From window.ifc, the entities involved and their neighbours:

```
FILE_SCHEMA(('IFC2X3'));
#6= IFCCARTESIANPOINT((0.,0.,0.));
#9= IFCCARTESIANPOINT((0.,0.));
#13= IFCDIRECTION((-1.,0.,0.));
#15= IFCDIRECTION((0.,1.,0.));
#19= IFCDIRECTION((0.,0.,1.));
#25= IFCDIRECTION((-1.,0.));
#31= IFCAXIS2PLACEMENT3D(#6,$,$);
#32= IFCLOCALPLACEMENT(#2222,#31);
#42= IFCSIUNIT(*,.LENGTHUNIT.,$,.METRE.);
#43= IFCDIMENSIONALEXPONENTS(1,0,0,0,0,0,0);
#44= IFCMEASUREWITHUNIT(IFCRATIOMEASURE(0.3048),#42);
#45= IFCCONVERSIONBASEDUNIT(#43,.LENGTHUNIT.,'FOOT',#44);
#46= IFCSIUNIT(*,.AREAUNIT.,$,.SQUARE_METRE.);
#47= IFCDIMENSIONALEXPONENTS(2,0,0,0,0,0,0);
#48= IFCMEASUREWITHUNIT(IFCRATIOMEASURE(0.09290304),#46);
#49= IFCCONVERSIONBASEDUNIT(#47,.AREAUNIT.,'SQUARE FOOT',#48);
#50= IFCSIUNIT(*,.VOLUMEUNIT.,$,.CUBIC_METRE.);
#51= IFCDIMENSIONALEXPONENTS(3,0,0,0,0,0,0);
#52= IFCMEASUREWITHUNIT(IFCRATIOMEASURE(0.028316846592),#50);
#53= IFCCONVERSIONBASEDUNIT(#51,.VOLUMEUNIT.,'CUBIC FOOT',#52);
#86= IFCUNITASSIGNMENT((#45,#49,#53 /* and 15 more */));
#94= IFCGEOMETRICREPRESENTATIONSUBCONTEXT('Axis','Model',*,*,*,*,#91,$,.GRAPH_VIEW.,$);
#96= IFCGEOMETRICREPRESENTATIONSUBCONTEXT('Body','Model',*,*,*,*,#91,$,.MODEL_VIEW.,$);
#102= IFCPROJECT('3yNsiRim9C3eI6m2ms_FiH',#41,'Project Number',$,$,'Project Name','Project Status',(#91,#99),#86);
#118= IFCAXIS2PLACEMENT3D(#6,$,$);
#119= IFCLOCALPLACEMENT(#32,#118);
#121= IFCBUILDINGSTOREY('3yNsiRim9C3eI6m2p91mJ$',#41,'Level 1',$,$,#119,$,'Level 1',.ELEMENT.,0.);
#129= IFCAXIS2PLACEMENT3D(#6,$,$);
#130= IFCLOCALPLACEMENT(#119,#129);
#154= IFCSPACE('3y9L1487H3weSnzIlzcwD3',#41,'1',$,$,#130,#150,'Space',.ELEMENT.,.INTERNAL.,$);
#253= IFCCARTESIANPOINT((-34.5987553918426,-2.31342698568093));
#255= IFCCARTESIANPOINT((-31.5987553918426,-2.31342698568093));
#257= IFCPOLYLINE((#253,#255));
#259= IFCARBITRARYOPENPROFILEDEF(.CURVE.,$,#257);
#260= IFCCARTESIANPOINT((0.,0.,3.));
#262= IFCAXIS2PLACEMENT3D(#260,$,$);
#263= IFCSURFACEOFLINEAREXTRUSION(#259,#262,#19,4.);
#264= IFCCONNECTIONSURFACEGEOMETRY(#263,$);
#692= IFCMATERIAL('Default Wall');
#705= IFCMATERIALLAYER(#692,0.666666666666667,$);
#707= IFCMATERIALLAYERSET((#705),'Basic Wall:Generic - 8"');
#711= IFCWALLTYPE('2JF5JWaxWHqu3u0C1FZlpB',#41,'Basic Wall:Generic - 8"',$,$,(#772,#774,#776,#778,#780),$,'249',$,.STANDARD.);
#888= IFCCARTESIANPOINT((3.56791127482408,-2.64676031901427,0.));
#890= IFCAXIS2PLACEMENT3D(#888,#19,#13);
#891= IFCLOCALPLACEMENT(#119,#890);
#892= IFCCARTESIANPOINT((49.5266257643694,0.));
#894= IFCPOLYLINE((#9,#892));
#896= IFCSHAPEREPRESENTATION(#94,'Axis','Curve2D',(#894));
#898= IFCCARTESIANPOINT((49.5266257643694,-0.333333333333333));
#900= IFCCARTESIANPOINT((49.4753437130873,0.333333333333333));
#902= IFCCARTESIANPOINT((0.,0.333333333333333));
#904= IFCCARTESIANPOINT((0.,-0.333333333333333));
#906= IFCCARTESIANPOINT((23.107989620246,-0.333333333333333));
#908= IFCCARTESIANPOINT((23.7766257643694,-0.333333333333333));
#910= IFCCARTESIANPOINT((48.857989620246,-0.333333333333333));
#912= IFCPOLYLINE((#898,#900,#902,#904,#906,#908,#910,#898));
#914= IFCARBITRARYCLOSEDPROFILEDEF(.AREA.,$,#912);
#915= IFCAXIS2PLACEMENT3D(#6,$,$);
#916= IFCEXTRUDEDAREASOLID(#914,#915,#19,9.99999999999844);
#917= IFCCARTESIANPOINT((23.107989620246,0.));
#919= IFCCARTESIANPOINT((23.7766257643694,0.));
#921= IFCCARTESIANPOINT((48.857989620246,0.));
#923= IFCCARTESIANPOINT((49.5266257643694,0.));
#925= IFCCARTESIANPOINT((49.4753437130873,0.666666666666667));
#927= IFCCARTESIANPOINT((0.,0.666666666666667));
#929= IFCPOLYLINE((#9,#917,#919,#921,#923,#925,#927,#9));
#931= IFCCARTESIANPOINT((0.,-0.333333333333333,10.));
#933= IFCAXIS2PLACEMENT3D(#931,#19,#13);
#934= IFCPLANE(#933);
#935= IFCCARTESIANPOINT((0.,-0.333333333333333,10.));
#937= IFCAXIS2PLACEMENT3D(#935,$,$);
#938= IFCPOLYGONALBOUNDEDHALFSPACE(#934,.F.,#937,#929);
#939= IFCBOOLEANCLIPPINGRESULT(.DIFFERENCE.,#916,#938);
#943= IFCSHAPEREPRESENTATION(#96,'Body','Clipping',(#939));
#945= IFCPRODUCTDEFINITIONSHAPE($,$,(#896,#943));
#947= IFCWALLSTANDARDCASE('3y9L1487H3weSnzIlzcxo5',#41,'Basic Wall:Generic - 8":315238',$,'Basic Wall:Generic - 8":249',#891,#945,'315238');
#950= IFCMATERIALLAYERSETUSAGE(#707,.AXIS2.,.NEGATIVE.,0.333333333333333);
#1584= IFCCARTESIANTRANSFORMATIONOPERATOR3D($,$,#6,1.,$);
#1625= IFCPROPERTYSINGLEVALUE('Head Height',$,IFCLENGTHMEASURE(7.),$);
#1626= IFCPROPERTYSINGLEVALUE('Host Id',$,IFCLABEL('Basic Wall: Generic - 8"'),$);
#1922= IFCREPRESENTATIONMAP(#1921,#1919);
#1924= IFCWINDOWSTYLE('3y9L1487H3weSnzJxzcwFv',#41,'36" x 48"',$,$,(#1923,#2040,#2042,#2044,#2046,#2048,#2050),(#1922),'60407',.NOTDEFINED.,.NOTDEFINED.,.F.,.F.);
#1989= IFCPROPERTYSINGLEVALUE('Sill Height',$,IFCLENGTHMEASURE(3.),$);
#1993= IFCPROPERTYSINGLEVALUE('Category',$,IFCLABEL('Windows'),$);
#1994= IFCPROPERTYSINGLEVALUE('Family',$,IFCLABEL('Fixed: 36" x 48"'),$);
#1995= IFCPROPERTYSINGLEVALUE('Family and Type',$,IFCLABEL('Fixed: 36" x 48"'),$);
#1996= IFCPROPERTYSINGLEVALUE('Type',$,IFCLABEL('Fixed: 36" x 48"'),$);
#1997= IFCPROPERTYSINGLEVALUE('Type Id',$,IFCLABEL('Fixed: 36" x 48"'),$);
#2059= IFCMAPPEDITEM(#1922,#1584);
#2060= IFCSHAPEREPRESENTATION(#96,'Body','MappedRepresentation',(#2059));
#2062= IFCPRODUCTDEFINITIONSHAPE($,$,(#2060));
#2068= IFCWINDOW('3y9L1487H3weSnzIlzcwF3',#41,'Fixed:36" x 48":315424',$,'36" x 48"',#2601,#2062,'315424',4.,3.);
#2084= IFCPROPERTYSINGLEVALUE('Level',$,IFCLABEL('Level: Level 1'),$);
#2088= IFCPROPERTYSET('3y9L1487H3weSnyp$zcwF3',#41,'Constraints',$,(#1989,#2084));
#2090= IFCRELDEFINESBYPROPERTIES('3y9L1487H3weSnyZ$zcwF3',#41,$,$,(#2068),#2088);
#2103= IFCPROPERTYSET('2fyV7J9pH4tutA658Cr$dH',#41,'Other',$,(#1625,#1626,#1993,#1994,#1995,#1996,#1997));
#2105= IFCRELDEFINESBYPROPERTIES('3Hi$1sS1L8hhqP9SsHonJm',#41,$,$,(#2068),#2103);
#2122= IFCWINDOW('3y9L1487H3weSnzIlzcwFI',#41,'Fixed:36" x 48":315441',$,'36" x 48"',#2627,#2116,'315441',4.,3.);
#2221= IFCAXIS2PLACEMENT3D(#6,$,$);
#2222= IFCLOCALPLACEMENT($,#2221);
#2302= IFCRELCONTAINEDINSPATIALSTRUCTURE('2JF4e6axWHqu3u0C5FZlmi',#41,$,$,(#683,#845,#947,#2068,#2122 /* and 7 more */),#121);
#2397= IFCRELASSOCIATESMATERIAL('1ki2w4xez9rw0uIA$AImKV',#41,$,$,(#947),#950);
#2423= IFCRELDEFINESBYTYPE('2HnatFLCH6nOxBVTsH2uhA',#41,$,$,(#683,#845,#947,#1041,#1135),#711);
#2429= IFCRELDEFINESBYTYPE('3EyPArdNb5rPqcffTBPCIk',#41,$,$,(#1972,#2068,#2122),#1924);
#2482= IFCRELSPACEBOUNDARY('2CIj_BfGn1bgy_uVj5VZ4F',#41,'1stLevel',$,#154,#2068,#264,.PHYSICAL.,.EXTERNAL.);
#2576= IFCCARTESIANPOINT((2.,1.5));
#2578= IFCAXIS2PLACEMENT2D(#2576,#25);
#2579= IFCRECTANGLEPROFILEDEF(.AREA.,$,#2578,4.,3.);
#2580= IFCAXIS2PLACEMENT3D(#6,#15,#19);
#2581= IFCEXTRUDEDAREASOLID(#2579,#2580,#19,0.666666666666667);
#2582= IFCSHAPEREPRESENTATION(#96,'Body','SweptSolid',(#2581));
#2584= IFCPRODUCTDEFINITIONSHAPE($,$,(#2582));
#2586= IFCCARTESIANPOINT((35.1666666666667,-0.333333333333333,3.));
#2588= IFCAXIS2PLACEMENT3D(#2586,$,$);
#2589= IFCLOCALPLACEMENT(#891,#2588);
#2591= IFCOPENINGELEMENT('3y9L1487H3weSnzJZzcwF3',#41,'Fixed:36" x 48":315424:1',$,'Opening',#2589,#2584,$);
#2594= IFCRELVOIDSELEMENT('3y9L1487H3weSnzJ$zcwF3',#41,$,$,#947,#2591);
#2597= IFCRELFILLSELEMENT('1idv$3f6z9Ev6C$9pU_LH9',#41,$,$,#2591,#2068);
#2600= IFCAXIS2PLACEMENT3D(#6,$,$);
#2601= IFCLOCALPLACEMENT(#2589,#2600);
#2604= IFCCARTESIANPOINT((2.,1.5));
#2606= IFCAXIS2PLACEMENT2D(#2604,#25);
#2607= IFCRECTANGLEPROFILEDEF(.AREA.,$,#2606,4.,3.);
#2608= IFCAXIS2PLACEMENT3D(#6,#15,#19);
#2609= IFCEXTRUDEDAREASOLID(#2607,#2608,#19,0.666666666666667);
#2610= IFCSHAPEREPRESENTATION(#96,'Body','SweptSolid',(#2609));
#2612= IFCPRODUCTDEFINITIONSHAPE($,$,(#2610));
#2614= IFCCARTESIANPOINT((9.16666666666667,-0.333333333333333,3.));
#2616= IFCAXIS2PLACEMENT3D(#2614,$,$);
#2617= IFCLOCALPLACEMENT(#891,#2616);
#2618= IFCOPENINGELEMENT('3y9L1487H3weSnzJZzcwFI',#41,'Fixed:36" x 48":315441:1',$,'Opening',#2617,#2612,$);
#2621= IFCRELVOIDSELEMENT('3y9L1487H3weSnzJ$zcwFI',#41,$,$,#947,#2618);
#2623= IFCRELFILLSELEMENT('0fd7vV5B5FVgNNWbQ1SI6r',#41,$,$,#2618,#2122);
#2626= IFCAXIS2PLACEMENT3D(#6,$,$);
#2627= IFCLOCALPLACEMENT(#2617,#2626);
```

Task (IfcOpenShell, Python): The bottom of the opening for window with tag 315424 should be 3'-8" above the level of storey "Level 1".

```python
import numpy as np
import ifcopenshell
import ifcopenshell.api.geometry
import ifcopenshell.api.pset
import ifcopenshell.geom
import ifcopenshell.util.element
import ifcopenshell.util.placement
import ifcopenshell.util.shape
import ifcopenshell.util.unit

model = ifcopenshell.open("window.ifc")
unit_scale = ifcopenshell.util.unit.calculate_unit_scale(model)

window = model.by_guid("3y9L1487H3weSnzIlzcwF3")
opening = window.FillsVoids[0].RelatingOpeningElement
storey = ifcopenshell.util.element.get_container(window, ifc_class="IfcBuildingStorey")
level = ifcopenshell.util.placement.get_local_placement(storey.ObjectPlacement)[2, 3]

# The opening's origin need not be at the sill, so measure its lowest point.
shape = ifcopenshell.geom.create_shape(ifcopenshell.geom.settings(), opening)
bottom = ifcopenshell.util.shape.get_shape_bottom_elevation(shape, shape.geometry) / unit_scale
dz = level + 44 * 0.0254 / unit_scale - bottom

shift = np.array([0.0, 0.0, dz])
# The window is placed relative to its opening, so it follows when the opening moves.
matrix = ifcopenshell.util.placement.get_local_placement(opening.ObjectPlacement)
matrix[:3, 3] += shift
ifcopenshell.api.geometry.edit_object_placement(
    model, product=opening, matrix=matrix, is_si=False, should_transform_children=True
)

# Space boundary surfaces are stored in each space's coordinates; move them too.
for rel in window.ProvidesBoundaries:
    if not rel.ConnectionGeometry:
        continue
    surface = rel.ConnectionGeometry.SurfaceOnRelatingElement
    space_matrix = ifcopenshell.util.placement.get_local_placement(rel.RelatingSpace.ObjectPlacement)
    point = np.array(surface.Position.Location.Coordinates) + space_matrix[:3, :3].T @ shift
    surface.Position = model.createIfcAxis2Placement3D(
        model.createIfcCartesianPoint(point.tolist()), surface.Position.Axis, surface.Position.RefDirection
    )

# Keep the stored heights in step.
pset = model.by_id(ifcopenshell.util.element.get_pset(window, "Constraints", should_inherit=False)["id"])
ifcopenshell.api.pset.edit_pset(model, pset=pset, properties={
    "Sill Height": model.create_entity("IfcLengthMeasure", ifcopenshell.util.element.get_pset(window, "Constraints", "Sill Height") + dz),
})
pset = model.by_id(ifcopenshell.util.element.get_pset(window, "Other", should_inherit=False)["id"])
ifcopenshell.api.pset.edit_pset(model, pset=pset, properties={
    "Head Height": model.create_entity("IfcLengthMeasure", ifcopenshell.util.element.get_pset(window, "Other", "Head Height") + dz),
})

print(f"moved by {dz * unit_scale:+.3f} m")

model.write("window_edited.ifc")
```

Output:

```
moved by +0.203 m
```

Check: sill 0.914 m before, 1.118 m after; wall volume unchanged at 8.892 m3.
